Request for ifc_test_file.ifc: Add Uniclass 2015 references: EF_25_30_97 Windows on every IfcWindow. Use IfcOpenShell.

First a look at what the model holds.

```python
import ifcopenshell

model = ifcopenshell.open("ifc_test_file.ifc")
print(model.schema)
print("classifications:", [c.Name for c in model.by_type("IfcClassification")])
for ifc_class in ("IfcDoor", "IfcRoof", "IfcStair", "IfcWall", "IfcWindow"):
    print(ifc_class, len(model.by_type(ifc_class)))
```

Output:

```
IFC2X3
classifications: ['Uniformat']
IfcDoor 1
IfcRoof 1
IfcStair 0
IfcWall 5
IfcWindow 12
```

```python
import ifcopenshell
import ifcopenshell.api.classification

model = ifcopenshell.open("ifc_test_file.ifc")

# IFC2X3 requires Source and Edition and has no link from the project to the system.
system = model.create_entity("IfcClassification", Source="NBS", Edition="2015", Name="Uniclass 2015")

codes = {
    "IfcWindow": ("EF_25_30_97", "Windows"),
}
for ifc_class, (code, name) in codes.items():
    products = model.by_type(ifc_class)
    ifcopenshell.api.classification.add_reference(
        model, products=products, classification=system, identification=code, name=name
    )
    print(code, len(products))

model.write("ifc_test_file_updated.ifc")
```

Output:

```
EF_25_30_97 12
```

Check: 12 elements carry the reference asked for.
